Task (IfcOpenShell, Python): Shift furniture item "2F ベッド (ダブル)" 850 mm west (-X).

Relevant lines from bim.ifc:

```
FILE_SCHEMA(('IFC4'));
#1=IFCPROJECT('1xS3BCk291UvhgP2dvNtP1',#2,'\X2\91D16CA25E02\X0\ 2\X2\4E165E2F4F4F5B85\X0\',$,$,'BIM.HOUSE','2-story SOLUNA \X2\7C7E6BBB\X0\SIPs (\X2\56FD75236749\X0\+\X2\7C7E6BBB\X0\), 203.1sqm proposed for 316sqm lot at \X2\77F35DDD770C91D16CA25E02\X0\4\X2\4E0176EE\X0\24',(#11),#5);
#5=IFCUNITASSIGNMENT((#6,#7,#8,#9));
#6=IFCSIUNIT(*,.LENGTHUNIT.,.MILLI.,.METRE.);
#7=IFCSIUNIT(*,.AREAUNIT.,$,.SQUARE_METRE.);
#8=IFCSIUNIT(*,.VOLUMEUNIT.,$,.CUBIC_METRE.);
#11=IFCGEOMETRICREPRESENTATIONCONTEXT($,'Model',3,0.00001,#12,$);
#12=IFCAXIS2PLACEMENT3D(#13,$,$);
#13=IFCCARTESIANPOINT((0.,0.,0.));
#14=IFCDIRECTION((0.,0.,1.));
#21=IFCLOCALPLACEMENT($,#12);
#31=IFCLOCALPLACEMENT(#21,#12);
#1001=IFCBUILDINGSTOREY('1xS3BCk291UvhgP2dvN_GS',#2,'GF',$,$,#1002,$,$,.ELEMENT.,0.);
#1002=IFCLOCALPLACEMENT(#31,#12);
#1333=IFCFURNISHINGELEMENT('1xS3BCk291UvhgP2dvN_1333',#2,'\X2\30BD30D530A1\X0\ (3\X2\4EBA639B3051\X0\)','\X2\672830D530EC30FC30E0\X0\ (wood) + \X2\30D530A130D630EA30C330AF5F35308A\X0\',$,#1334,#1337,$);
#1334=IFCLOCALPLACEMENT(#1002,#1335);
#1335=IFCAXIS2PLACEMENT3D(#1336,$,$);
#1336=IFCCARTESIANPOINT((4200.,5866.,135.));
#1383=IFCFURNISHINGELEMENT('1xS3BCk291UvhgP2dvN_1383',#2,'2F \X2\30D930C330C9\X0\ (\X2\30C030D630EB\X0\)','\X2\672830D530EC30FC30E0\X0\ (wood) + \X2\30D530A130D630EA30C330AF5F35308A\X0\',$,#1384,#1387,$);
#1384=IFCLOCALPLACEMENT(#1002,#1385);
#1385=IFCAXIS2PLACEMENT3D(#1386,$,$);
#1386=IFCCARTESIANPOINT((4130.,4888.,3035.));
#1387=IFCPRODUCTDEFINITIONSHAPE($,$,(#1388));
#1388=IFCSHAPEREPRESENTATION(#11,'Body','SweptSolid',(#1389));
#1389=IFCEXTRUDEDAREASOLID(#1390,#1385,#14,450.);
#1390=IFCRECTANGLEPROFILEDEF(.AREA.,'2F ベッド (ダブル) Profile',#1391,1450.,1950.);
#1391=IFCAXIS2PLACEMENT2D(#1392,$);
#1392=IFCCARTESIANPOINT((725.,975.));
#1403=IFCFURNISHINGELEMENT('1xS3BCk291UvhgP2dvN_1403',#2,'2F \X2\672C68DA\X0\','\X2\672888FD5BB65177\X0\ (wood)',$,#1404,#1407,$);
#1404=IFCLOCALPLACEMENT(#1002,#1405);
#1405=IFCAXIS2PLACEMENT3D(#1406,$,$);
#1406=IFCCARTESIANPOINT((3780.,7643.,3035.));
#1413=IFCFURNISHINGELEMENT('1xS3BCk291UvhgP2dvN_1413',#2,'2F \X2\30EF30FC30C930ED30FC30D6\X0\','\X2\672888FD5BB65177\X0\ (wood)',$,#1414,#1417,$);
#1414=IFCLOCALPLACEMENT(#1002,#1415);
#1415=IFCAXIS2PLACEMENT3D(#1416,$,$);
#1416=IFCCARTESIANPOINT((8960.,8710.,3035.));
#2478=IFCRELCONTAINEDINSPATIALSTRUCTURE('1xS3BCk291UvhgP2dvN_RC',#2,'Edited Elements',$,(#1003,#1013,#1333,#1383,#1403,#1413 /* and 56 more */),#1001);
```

```python
import ifcopenshell
import ifcopenshell.api.geometry
import ifcopenshell.util.placement
import ifcopenshell.util.unit

model = ifcopenshell.open("bim.ifc")
unit_scale = ifcopenshell.util.unit.calculate_unit_scale(model)

item = model.by_id(1383)
matrix = ifcopenshell.util.placement.get_local_placement(item.ObjectPlacement)
matrix[0, 3] -= 0.85 / unit_scale
ifcopenshell.api.geometry.edit_object_placement(model, product=item, matrix=matrix, is_si=False)

print(ifcopenshell.util.placement.get_local_placement(item.ObjectPlacement).round(3) + 0.0)

model.write("bim-out.ifc")
```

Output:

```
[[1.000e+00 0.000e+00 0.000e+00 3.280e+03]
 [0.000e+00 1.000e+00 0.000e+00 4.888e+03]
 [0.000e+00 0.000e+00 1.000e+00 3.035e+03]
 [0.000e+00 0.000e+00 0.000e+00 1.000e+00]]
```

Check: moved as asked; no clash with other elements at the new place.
